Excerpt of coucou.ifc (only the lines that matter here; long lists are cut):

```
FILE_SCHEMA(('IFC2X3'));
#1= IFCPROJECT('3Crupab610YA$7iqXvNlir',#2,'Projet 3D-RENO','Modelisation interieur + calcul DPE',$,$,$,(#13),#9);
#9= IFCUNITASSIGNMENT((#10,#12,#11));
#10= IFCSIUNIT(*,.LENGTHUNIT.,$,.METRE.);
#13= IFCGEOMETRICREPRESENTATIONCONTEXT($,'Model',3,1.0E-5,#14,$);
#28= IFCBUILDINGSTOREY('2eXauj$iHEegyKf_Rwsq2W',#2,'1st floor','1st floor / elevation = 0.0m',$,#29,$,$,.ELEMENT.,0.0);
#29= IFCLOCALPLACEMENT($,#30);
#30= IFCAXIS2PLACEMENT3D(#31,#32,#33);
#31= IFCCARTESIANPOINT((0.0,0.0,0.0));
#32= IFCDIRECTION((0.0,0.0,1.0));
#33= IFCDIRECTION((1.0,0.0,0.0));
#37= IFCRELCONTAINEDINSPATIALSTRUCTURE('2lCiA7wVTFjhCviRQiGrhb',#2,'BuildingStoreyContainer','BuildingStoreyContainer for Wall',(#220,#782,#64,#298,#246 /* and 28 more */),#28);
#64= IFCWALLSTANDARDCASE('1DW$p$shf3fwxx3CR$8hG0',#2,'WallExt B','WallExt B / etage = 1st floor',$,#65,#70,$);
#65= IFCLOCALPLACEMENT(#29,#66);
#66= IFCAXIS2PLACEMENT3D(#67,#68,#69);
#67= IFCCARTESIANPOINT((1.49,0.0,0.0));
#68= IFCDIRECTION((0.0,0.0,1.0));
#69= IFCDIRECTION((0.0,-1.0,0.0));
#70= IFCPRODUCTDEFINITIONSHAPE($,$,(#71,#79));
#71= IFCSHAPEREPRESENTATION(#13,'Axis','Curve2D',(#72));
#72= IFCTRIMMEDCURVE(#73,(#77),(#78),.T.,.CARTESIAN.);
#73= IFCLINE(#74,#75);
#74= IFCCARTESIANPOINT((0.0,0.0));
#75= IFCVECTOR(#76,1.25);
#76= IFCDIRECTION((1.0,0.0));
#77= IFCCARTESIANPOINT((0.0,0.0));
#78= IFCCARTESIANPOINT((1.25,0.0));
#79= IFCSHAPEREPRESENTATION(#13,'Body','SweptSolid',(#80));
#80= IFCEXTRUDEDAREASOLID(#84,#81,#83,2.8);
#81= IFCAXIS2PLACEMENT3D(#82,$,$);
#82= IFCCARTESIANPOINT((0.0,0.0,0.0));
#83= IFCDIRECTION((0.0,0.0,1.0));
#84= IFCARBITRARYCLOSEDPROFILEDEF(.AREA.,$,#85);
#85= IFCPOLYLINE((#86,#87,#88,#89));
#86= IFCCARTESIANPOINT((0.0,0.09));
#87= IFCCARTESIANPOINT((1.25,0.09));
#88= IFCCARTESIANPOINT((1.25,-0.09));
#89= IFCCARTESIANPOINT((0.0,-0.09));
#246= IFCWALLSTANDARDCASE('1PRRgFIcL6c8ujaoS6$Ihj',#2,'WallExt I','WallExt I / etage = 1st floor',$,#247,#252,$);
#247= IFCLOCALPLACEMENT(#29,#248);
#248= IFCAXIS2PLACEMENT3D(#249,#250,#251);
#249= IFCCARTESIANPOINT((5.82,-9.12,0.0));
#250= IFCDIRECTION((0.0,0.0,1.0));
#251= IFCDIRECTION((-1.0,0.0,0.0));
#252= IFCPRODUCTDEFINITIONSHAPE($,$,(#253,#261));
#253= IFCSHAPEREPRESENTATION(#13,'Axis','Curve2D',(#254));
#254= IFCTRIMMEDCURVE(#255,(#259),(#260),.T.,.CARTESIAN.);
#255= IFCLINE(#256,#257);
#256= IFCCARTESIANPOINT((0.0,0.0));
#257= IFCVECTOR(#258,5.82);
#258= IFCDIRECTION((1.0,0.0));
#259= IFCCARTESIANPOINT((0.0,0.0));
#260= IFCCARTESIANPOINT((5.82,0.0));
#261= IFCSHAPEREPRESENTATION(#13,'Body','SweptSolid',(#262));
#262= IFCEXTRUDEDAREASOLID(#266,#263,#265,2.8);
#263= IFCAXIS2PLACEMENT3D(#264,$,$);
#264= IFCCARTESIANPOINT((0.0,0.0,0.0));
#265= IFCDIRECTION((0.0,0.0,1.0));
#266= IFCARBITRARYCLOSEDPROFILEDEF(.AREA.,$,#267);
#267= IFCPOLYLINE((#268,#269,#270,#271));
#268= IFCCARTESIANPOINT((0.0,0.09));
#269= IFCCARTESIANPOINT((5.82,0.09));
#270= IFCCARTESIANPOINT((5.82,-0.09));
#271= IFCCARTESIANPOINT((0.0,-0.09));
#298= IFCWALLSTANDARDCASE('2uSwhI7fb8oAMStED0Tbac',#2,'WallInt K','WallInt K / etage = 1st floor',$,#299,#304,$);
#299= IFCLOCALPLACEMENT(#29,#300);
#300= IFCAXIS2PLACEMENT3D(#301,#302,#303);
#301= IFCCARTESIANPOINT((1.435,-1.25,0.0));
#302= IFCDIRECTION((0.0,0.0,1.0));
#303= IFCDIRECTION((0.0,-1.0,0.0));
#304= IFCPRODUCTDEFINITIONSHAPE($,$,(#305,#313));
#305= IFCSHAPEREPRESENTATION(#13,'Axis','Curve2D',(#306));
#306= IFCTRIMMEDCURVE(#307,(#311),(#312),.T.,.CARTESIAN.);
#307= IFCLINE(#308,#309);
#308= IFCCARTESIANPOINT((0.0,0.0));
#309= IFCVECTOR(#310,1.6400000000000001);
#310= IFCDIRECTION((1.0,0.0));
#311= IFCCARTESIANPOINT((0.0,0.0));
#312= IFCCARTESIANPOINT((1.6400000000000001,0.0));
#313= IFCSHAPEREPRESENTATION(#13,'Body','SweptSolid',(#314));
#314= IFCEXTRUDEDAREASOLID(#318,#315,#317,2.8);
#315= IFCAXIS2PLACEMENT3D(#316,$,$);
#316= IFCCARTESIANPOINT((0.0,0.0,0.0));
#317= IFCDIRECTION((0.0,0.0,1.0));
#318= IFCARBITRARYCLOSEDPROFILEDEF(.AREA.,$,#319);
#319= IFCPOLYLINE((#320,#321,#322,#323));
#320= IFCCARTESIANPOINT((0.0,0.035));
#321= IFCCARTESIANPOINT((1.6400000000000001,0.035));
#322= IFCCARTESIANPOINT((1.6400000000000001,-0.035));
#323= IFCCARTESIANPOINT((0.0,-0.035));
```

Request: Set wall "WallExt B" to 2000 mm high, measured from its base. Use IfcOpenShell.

```python
import ifcopenshell
import ifcopenshell.geom
import ifcopenshell.util.shape
import ifcopenshell.util.unit

model = ifcopenshell.open("coucou.ifc")
unit_scale = ifcopenshell.util.unit.calculate_unit_scale(model)
settings = ifcopenshell.geom.settings()


def volume(element):
    """Net volume in cubic metres, openings subtracted."""
    shape = ifcopenshell.geom.create_shape(settings, element)
    return ifcopenshell.util.shape.get_volume(shape.geometry)


wall = model.by_guid("1DW$p$shf3fwxx3CR$8hG0")
before = volume(wall)

body = next(r for r in wall.Representation.Representations if r.RepresentationIdentifier == "Body")
solid = body.Items[0]
old_height = solid.Depth
solid.Depth = 2 / unit_scale
after = volume(wall)

print(f"height {old_height:g} -> {solid.Depth:g}, volume {before:.3f} -> {after:.3f} m3")

model.write("coucou_edited.ifc")
```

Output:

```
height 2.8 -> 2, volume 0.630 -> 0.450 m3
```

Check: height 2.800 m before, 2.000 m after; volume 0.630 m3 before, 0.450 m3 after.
